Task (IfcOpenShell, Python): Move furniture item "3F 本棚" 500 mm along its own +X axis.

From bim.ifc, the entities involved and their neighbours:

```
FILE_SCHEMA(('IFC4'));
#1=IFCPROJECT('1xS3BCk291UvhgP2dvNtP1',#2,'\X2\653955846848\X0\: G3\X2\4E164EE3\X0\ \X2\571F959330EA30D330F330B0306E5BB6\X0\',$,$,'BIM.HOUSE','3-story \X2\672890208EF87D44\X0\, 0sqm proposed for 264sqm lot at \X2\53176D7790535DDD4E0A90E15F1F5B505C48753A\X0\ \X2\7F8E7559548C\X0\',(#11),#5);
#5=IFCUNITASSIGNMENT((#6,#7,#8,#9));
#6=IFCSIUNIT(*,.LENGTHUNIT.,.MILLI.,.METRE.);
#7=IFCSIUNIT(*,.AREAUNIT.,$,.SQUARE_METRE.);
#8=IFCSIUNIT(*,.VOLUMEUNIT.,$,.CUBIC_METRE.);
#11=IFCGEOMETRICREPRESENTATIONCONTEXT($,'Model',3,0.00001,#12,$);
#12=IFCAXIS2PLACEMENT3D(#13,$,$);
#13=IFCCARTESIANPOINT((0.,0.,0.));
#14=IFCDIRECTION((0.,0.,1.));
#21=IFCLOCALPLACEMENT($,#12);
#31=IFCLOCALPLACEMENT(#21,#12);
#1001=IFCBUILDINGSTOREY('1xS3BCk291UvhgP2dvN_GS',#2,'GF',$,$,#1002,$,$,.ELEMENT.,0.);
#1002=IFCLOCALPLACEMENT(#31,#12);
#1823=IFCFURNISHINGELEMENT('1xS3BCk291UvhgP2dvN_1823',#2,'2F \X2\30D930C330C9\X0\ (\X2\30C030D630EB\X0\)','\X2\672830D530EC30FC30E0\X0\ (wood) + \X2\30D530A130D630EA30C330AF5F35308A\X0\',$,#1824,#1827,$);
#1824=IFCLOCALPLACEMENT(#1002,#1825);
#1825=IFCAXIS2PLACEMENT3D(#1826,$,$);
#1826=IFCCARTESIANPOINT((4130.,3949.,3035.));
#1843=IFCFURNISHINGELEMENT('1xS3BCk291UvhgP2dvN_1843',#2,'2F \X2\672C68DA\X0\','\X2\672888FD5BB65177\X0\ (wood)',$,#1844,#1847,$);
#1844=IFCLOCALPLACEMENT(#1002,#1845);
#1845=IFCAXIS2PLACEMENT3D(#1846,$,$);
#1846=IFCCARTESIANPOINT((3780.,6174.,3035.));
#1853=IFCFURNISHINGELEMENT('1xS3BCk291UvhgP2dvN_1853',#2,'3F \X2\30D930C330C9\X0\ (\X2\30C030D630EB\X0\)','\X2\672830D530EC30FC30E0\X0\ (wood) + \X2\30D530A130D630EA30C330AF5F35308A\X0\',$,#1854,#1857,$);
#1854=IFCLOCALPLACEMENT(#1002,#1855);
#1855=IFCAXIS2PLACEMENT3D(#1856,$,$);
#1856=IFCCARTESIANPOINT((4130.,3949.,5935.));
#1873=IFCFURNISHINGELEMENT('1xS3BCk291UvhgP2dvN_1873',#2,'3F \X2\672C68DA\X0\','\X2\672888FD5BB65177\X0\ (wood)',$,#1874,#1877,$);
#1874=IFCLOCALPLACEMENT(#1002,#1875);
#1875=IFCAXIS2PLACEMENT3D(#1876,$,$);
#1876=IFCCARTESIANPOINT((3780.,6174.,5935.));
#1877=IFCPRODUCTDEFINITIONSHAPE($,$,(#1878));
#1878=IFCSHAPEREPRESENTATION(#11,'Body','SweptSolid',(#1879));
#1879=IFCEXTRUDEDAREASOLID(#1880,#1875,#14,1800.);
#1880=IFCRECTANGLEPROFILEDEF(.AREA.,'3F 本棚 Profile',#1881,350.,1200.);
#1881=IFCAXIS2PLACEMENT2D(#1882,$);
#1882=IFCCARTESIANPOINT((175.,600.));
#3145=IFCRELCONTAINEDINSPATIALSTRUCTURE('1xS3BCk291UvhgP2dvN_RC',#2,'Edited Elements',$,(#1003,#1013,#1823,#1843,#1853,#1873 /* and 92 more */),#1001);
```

```python
import ifcopenshell
import ifcopenshell.api.geometry
import ifcopenshell.util.placement

model = ifcopenshell.open("bim.ifc")

item = model.by_guid("1xS3BCk291UvhgP2dvN_1873")
matrix = ifcopenshell.util.placement.get_local_placement(item.ObjectPlacement)
matrix[:3, 3] += matrix[:3, 0] * 500.0
ifcopenshell.api.geometry.edit_object_placement(model, product=item, matrix=matrix, is_si=False)

print(ifcopenshell.util.placement.get_local_placement(item.ObjectPlacement).round(3) + 0.0)

model.write("bim_edited.ifc")
```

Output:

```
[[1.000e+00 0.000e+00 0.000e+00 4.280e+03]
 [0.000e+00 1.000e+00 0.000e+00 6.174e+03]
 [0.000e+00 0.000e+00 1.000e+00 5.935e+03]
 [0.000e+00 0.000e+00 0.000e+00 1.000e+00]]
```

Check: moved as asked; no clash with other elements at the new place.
